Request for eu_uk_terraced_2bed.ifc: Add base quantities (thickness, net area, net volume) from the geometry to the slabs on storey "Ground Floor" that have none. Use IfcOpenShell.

First a look at what the model holds.

```python
import ifcopenshell
import ifcopenshell.util.element
import ifcopenshell.util.unit

model = ifcopenshell.open("eu_uk_terraced_2bed.ifc")
print(model.schema)
for unit_type in ("LENGTHUNIT", "AREAUNIT", "VOLUMEUNIT"):
    print(unit_type, ifcopenshell.util.unit.calculate_unit_scale(model, unit_type))
storey = next(s for s in model.by_type("IfcBuildingStorey") if s.Name == "Ground Floor")
slabs = [e for e in ifcopenshell.util.element.get_decomposition(storey) if e.is_a("IfcSlab")]
for e in sorted(slabs, key=lambda e: e.id()):
    print(e.id(), e.is_a(), e.Name, list(ifcopenshell.util.element.get_psets(e, qtos_only=True)), sep=" | ")
```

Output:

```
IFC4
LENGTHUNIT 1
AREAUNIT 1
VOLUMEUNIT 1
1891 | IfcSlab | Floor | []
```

```python
import ifcopenshell
import ifcopenshell.api.pset
import ifcopenshell.geom
import ifcopenshell.util.element
import ifcopenshell.util.shape
import ifcopenshell.util.unit

model = ifcopenshell.open("eu_uk_terraced_2bed.ifc")
unit_scale = ifcopenshell.util.unit.calculate_unit_scale(model)
area_scale = ifcopenshell.util.unit.calculate_unit_scale(model, "AREAUNIT")
volume_scale = ifcopenshell.util.unit.calculate_unit_scale(model, "VOLUMEUNIT")
settings = ifcopenshell.geom.settings()

storey = next(s for s in model.by_type("IfcBuildingStorey") if s.Name == "Ground Floor")
slabs = [e for e in ifcopenshell.util.element.get_decomposition(storey) if e.is_a("IfcSlab")]

for e in sorted(slabs, key=lambda e: e.id()):
    if ifcopenshell.util.element.get_psets(e, qtos_only=True, should_inherit=False):
        continue
    # Geometry comes back in metres, in the element's own axes.
    shape = ifcopenshell.geom.create_shape(settings, e)
    values = {
        "Width": ifcopenshell.util.shape.get_z(shape.geometry) / unit_scale,
        "NetArea": ifcopenshell.util.shape.get_footprint_area(shape.geometry) / area_scale,
        "NetVolume": ifcopenshell.util.shape.get_volume(shape.geometry) / volume_scale,
    }
    qto = ifcopenshell.api.pset.add_qto(model, product=e, name="Qto_SlabBaseQuantities")
    ifcopenshell.api.pset.edit_qto(model, qto=qto, properties=values)
    print(e.id(), {k: round(v, 3) for k, v in values.items()})

model.write("eu_uk_terraced_2bed_v2.ifc")
```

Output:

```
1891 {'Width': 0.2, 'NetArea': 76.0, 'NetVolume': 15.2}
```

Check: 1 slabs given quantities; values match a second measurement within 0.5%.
